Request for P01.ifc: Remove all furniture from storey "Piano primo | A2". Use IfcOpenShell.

First a look at what the model holds.

```python
import ifcopenshell
import ifcopenshell.util.element

model = ifcopenshell.open("P01.ifc")
print(model.schema)
storey = next(s for s in model.by_type("IfcBuildingStorey") if s.Name == "Piano primo | A2")
furniture = [e for e in ifcopenshell.util.element.get_decomposition(storey) if e.is_a("IfcFurnishingElement")]
seen = {}
for e in furniture:
    element_type = ifcopenshell.util.element.get_type(e)
    name = element_type.Name if element_type not in (None, e) else None
    seen[name] = seen.get(name, 0) + 1
for name, count in sorted(seen.items(), key=str):
    print(count, "x", name)
```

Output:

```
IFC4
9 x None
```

```python
import ifcopenshell
import ifcopenshell.api.root
import ifcopenshell.util.element

model = ifcopenshell.open("P01.ifc")

storey = next(s for s in model.by_type("IfcBuildingStorey") if s.Name == "Piano primo | A2")
furniture = [e for e in ifcopenshell.util.element.get_decomposition(storey) if e.is_a("IfcFurnishingElement")]

for e in furniture:
    ifcopenshell.api.root.remove_product(model, product=e)
print(len(furniture), "removed")

model.write("P01_v2.ifc")
```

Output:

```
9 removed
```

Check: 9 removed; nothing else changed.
